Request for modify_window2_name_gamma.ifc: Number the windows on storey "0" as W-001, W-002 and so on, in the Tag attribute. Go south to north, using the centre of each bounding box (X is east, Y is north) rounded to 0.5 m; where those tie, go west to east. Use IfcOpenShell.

First a look at what the model holds.

```python
import ifcopenshell
import ifcopenshell.util.element
import ifcopenshell.util.placement

model = ifcopenshell.open("modify_window2_name_gamma.ifc")
print(model.schema)
storey = next(s for s in model.by_type("IfcBuildingStorey") if s.Name == "0")
windows = [e for e in ifcopenshell.util.element.get_decomposition(storey) if e.is_a("IfcWindow")]
for e in sorted(windows, key=lambda e: e.id()):
    origin = ifcopenshell.util.placement.get_local_placement(e.ObjectPlacement)[:3, 3]
    print(e.id(), e.Tag, e.Name, origin.round(2) + 0.0, sep=" | ")
```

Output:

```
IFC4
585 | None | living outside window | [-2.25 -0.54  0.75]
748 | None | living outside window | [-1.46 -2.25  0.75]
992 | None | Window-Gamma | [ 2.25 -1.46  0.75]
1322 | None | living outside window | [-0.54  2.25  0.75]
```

```python
import ifcopenshell
import ifcopenshell.geom
import ifcopenshell.util.element
import ifcopenshell.util.shape

model = ifcopenshell.open("modify_window2_name_gamma.ifc")
settings = ifcopenshell.geom.settings()
settings.set("use-world-coords", True)


def centre(element):
    shape = ifcopenshell.geom.create_shape(settings, element)
    return ifcopenshell.util.shape.get_bbox_centroid(shape.geometry)


storey = next(s for s in model.by_type("IfcBuildingStorey") if s.Name == "0")
windows = [e for e in ifcopenshell.util.element.get_decomposition(storey) if e.is_a("IfcWindow")]

# Insertion points can sit at a corner or the storey origin, so sort by the geometry (in metres).
centres = {e: centre(e) for e in windows}
windows.sort(key=lambda e: (round(centres[e][1] / 0.5), centres[e][0]))

for i, e in enumerate(windows, start=1):
    number = f"W-0{i:02d}"
    e.Tag = number
    print(e.id(), number)

model.write("modify_window2_name_gamma_updated.ifc")
```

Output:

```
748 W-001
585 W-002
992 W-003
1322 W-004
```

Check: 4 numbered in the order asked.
